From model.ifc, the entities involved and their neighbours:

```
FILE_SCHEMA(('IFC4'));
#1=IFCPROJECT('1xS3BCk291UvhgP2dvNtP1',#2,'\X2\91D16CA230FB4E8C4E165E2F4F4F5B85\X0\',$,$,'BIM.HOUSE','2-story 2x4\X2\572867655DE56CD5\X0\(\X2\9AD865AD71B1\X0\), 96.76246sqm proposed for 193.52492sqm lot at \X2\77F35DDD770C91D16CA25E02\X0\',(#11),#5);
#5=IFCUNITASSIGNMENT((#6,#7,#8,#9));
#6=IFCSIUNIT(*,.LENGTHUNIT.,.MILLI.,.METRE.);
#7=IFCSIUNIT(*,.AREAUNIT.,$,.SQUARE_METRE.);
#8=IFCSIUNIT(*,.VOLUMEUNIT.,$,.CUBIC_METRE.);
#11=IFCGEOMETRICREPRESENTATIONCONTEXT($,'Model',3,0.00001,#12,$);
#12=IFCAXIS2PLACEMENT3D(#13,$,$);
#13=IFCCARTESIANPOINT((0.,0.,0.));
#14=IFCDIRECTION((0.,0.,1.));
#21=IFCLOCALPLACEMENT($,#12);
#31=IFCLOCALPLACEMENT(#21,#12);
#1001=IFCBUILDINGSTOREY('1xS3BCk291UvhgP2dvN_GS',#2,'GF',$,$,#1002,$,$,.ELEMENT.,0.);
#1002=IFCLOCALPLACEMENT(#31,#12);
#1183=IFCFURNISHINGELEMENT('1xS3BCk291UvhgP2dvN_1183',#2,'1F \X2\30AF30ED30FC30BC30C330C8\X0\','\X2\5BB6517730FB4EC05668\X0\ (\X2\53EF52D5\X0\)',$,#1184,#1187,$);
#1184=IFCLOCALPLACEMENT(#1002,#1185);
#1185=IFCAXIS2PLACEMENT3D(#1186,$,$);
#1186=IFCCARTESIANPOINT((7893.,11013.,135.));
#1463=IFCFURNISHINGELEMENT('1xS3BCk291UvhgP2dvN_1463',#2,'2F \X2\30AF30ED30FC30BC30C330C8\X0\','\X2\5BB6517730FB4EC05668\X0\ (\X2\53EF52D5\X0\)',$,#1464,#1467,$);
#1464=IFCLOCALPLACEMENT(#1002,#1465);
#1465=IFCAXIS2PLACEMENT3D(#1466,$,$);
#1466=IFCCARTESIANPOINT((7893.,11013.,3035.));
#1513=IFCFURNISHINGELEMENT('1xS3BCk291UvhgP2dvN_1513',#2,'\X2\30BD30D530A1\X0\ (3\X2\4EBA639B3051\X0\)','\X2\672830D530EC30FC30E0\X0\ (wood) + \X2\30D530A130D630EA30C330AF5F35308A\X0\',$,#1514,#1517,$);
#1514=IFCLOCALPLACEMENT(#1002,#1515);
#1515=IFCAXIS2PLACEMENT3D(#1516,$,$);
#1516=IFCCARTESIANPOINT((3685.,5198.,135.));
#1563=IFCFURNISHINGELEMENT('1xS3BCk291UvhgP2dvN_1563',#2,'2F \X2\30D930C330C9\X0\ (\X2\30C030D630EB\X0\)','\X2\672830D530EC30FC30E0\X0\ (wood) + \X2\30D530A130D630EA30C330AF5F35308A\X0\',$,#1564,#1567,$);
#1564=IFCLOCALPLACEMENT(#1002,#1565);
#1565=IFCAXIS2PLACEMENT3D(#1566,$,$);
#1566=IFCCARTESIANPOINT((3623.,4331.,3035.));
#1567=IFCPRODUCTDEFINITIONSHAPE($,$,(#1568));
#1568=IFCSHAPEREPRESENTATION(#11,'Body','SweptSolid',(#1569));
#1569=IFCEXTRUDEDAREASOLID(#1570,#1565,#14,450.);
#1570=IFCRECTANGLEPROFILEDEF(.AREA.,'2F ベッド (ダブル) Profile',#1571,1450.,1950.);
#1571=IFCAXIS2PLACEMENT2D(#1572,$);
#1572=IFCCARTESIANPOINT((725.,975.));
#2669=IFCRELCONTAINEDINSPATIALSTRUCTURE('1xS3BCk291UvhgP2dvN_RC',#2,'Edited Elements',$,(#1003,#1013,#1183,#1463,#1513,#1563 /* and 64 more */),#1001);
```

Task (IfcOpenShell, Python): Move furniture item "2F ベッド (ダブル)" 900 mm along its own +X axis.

```python
import ifcopenshell
import ifcopenshell.api.geometry
import ifcopenshell.util.placement

model = ifcopenshell.open("model.ifc")

item = model.by_id(1563)
matrix = ifcopenshell.util.placement.get_local_placement(item.ObjectPlacement)
matrix[:3, 3] += matrix[:3, 0] * 900.0
ifcopenshell.api.geometry.edit_object_placement(model, product=item, matrix=matrix, is_si=False)

print(ifcopenshell.util.placement.get_local_placement(item.ObjectPlacement).round(3) + 0.0)

model.write("model_edited.ifc")
```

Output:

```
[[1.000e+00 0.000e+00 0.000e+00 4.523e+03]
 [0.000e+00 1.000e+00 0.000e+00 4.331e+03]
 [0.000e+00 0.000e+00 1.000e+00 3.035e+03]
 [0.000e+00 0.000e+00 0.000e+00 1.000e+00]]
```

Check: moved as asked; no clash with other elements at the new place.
